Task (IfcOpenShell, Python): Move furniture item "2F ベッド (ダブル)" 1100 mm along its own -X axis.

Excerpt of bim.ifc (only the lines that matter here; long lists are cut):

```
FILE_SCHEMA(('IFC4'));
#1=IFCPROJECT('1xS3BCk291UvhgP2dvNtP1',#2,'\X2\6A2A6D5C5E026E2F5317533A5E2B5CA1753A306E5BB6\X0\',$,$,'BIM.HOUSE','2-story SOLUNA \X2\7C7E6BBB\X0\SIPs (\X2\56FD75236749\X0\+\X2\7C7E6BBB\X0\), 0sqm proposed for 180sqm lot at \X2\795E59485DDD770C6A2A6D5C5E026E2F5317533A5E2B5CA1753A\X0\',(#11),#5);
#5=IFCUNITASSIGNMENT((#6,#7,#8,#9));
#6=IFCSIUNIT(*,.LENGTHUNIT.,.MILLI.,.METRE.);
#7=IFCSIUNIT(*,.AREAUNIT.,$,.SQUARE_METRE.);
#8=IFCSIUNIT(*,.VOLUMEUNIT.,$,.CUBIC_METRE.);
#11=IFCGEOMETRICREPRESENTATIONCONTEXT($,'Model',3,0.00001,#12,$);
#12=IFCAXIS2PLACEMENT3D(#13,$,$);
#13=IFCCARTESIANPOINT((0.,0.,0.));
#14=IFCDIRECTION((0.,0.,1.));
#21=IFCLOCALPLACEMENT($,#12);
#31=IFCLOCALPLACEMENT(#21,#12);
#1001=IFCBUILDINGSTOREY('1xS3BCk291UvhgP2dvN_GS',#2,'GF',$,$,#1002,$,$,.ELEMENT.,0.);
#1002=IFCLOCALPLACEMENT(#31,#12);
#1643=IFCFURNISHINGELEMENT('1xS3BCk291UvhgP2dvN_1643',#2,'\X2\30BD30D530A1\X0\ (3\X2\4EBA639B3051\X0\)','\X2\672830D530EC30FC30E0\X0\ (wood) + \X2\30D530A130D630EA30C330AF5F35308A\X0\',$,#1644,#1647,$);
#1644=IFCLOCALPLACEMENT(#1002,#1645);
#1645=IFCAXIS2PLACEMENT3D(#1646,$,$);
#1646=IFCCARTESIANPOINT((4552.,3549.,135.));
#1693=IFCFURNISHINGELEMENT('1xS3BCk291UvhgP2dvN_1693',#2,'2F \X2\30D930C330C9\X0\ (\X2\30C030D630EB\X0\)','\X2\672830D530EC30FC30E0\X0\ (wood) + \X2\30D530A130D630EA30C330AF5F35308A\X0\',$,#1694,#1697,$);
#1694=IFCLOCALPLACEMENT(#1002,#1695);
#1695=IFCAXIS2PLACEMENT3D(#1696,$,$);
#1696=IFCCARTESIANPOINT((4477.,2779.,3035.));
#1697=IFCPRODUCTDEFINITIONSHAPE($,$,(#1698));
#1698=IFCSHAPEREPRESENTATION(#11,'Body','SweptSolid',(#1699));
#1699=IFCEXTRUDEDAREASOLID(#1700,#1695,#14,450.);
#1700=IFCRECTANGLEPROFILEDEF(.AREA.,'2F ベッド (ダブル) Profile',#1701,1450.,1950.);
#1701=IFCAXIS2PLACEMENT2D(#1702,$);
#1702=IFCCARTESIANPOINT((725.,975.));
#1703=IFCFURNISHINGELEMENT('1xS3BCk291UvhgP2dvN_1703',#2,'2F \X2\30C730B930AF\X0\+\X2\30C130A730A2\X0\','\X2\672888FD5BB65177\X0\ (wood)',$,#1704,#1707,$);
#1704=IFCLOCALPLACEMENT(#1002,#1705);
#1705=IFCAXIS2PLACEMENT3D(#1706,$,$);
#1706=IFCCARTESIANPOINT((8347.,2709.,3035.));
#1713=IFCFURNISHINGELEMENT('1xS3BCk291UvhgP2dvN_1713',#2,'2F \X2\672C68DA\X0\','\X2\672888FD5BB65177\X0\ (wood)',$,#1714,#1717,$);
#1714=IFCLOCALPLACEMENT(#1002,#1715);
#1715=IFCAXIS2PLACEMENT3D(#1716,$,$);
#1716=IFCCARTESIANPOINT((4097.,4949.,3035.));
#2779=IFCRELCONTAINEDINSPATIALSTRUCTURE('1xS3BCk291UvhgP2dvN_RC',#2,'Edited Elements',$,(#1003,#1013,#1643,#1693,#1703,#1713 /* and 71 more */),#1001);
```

```python
import ifcopenshell
import ifcopenshell.api.geometry
import ifcopenshell.util.placement

model = ifcopenshell.open("bim.ifc")

item = model.by_guid("1xS3BCk291UvhgP2dvN_1693")
matrix = ifcopenshell.util.placement.get_local_placement(item.ObjectPlacement)
matrix[:3, 3] -= matrix[:3, 0] * 1100.0
ifcopenshell.api.geometry.edit_object_placement(model, product=item, matrix=matrix, is_si=False)

print(ifcopenshell.util.placement.get_local_placement(item.ObjectPlacement).round(3) + 0.0)

model.write("bim_v2.ifc")
```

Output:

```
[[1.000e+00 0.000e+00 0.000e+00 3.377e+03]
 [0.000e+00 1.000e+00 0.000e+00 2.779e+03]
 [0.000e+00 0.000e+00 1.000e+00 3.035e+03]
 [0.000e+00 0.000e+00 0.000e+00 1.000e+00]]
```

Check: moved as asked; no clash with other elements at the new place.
